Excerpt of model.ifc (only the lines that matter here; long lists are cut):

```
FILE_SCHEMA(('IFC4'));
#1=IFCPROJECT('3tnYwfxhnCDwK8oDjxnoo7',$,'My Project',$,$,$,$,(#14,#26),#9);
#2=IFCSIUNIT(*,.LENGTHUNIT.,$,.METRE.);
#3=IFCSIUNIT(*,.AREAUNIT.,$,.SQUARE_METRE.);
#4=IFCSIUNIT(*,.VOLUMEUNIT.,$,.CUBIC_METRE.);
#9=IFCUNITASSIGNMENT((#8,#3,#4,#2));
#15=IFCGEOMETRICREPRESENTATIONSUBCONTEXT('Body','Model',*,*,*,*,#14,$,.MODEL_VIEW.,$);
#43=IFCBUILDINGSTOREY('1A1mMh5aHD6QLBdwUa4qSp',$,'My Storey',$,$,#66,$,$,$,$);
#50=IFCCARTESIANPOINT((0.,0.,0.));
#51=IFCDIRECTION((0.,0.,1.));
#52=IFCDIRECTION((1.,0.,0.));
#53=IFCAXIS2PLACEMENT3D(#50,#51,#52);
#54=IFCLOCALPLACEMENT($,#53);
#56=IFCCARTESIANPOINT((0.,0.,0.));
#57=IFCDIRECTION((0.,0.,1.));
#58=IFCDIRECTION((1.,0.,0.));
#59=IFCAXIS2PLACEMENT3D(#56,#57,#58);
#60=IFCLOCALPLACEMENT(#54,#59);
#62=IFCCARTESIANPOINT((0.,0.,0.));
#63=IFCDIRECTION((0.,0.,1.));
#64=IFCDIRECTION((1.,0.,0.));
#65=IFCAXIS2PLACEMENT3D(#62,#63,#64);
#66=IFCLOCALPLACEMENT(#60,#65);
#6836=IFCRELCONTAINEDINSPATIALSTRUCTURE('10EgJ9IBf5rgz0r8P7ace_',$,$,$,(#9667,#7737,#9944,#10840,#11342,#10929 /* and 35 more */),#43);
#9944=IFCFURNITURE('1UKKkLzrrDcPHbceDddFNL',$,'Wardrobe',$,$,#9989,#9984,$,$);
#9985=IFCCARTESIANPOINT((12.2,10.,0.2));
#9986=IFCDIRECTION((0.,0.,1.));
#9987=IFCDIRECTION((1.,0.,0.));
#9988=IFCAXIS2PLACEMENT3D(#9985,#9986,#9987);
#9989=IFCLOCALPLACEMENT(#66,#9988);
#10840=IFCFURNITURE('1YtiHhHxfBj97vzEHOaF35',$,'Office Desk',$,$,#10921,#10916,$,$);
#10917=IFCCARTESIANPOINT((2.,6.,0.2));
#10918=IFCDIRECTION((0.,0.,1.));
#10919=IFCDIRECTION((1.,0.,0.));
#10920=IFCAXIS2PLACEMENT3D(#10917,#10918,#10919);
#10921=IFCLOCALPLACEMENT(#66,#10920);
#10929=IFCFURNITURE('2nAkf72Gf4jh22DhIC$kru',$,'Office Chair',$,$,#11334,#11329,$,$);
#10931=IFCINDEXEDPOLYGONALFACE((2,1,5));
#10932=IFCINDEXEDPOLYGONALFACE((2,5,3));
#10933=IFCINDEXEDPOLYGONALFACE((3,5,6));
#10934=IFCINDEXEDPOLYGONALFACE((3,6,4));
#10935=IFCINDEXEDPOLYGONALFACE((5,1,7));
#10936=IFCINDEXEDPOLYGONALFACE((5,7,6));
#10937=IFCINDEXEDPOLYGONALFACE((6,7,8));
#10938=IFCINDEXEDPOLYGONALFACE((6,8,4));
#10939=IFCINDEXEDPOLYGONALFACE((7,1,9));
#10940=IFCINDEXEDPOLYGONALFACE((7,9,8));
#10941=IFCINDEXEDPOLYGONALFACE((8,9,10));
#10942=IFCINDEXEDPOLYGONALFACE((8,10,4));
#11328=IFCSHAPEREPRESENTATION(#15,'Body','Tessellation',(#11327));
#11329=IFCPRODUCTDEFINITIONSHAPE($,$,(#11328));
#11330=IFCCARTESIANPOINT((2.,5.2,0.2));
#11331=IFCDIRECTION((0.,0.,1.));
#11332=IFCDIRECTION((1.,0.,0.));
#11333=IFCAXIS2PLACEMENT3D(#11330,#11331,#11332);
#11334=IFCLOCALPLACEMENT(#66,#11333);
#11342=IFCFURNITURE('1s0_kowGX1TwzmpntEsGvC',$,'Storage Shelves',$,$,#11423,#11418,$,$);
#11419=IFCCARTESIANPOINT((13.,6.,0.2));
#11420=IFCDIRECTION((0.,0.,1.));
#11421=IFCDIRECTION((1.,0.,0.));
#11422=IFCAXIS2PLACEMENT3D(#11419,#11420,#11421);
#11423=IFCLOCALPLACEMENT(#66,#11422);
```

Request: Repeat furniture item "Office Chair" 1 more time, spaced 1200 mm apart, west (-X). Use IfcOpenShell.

```python
import numpy as np
import ifcopenshell
import ifcopenshell.api.geometry
import ifcopenshell.api.root
import ifcopenshell.util.element
import ifcopenshell.util.placement
import ifcopenshell.util.unit

model = ifcopenshell.open("model.ifc")
unit_scale = ifcopenshell.util.unit.calculate_unit_scale(model)

source = model.by_id(10929)
base = ifcopenshell.util.placement.get_local_placement(source.ObjectPlacement)
step = np.array([-1.0, 0.0, 0.0]) * 1.2 / unit_scale

for i in range(1, 2):
    copy = ifcopenshell.api.root.copy_class(model, product=source)
    copy.Representation = ifcopenshell.util.element.copy_deep(
        model, source.Representation, exclude=["IfcGeometricRepresentationContext", "IfcRepresentationMap"]
    )
    matrix = base.copy()
    matrix[:3, 3] += i * step
    print("added at", matrix[:3, 3].round(3) + 0.0)
    ifcopenshell.api.geometry.edit_object_placement(model, product=copy, matrix=matrix, is_si=False)

model.write("model_v2.ifc")
```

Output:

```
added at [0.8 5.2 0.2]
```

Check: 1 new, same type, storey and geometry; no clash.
